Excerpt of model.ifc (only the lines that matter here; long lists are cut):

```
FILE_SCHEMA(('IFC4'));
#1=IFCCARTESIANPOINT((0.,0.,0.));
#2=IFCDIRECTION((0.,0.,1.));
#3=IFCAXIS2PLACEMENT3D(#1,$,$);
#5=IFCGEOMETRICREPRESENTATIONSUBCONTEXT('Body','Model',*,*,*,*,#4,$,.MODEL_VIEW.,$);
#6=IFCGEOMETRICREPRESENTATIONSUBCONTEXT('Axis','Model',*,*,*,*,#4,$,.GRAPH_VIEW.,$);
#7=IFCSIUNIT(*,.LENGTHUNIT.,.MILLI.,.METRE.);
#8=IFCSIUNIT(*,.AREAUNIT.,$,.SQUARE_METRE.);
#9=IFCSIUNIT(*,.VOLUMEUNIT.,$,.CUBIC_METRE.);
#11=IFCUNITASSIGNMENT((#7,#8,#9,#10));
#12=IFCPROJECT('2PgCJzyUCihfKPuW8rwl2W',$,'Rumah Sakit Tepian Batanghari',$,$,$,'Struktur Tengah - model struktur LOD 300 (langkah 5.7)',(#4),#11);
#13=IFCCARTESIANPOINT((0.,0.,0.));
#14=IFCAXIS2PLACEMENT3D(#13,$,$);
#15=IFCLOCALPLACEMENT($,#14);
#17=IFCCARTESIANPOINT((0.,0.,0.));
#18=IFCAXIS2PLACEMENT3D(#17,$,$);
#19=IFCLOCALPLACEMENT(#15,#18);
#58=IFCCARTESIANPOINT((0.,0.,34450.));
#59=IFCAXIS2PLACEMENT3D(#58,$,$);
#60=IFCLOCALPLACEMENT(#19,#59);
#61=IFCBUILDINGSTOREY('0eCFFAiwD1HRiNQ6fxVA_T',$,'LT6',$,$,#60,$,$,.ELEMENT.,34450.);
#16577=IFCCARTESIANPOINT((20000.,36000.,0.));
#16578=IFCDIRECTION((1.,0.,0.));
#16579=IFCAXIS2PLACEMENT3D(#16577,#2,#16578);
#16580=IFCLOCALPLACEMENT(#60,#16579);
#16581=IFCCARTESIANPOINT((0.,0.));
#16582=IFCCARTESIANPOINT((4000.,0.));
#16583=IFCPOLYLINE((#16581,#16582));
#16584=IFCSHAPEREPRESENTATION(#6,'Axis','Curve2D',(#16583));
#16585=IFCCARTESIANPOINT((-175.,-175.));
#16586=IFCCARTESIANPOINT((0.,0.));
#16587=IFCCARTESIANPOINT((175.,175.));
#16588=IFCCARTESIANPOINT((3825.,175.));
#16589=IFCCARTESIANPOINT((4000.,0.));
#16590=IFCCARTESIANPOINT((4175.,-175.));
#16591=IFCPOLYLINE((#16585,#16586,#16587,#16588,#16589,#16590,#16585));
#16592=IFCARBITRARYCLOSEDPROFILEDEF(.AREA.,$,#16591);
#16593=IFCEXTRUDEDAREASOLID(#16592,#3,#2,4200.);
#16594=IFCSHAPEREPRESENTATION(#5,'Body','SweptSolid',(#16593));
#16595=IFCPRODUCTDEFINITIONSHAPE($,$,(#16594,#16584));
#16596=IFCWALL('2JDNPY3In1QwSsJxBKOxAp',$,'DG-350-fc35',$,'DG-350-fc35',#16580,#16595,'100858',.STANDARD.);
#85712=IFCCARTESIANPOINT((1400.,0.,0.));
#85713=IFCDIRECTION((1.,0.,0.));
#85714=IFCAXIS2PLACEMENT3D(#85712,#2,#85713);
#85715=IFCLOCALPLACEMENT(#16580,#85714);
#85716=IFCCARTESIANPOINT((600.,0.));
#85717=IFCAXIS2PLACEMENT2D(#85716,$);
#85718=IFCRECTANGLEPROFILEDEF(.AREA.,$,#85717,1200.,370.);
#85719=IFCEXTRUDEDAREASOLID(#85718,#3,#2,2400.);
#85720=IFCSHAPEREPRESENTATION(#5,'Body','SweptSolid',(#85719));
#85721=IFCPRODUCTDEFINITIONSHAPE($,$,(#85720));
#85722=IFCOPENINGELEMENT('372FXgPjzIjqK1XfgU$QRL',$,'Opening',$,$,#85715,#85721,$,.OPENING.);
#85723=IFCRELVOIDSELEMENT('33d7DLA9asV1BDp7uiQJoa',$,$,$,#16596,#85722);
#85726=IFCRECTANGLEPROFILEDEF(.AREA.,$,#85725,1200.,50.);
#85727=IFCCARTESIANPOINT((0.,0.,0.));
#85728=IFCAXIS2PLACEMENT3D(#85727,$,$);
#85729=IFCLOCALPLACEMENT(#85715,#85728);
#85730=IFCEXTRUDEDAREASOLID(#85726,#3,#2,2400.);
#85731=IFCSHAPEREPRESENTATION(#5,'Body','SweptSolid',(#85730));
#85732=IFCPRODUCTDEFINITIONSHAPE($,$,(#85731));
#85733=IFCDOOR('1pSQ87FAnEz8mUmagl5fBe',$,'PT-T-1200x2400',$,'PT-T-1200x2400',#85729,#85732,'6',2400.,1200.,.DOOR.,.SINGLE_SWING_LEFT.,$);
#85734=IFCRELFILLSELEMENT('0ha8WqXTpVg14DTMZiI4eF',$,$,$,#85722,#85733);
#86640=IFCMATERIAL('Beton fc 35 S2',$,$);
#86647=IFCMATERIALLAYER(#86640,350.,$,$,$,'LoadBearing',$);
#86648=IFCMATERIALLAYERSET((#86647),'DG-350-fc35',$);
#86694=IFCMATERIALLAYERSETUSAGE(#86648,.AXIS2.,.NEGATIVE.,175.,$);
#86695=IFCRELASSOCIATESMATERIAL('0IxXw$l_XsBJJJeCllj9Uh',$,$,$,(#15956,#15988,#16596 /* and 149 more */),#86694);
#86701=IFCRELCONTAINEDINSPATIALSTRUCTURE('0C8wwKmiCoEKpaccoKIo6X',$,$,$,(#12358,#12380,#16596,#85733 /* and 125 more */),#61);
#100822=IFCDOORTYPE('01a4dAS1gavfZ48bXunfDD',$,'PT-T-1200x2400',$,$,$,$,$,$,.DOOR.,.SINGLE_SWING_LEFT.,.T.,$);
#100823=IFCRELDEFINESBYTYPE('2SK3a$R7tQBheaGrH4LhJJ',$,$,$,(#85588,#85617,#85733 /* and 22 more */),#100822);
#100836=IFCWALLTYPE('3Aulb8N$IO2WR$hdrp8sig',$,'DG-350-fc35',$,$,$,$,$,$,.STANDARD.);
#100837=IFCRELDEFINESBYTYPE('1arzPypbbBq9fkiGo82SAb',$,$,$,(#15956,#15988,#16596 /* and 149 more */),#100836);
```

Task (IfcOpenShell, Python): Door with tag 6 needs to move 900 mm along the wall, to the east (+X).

```python
import ifcopenshell
import ifcopenshell.api.geometry
import ifcopenshell.util.placement
import ifcopenshell.util.unit

model = ifcopenshell.open("model.ifc")
unit_scale = ifcopenshell.util.unit.calculate_unit_scale(model)

door = model.by_id(85733)
opening = door.FillsVoids[0].RelatingOpeningElement
wall = opening.VoidsElements[0].RelatingBuildingElement

wall_matrix = ifcopenshell.util.placement.get_local_placement(wall.ObjectPlacement)
shift = wall_matrix[:3, 0] * 0.9 / unit_scale
before = ifcopenshell.util.placement.get_local_placement(door.ObjectPlacement)[:3, 3].copy()

# The door is placed relative to its opening, so it follows when the opening moves.
matrix = ifcopenshell.util.placement.get_local_placement(opening.ObjectPlacement)
matrix[:3, 3] += shift
ifcopenshell.api.geometry.edit_object_placement(
    model, product=opening, matrix=matrix, is_si=False, should_transform_children=True
)

after = ifcopenshell.util.placement.get_local_placement(door.ObjectPlacement)[:3, 3]
print("door moved by", (after - before).round(3) + 0.0)

model.write("model_updated.ifc")
```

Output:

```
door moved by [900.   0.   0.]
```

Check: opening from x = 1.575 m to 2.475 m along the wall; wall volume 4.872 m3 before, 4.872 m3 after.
